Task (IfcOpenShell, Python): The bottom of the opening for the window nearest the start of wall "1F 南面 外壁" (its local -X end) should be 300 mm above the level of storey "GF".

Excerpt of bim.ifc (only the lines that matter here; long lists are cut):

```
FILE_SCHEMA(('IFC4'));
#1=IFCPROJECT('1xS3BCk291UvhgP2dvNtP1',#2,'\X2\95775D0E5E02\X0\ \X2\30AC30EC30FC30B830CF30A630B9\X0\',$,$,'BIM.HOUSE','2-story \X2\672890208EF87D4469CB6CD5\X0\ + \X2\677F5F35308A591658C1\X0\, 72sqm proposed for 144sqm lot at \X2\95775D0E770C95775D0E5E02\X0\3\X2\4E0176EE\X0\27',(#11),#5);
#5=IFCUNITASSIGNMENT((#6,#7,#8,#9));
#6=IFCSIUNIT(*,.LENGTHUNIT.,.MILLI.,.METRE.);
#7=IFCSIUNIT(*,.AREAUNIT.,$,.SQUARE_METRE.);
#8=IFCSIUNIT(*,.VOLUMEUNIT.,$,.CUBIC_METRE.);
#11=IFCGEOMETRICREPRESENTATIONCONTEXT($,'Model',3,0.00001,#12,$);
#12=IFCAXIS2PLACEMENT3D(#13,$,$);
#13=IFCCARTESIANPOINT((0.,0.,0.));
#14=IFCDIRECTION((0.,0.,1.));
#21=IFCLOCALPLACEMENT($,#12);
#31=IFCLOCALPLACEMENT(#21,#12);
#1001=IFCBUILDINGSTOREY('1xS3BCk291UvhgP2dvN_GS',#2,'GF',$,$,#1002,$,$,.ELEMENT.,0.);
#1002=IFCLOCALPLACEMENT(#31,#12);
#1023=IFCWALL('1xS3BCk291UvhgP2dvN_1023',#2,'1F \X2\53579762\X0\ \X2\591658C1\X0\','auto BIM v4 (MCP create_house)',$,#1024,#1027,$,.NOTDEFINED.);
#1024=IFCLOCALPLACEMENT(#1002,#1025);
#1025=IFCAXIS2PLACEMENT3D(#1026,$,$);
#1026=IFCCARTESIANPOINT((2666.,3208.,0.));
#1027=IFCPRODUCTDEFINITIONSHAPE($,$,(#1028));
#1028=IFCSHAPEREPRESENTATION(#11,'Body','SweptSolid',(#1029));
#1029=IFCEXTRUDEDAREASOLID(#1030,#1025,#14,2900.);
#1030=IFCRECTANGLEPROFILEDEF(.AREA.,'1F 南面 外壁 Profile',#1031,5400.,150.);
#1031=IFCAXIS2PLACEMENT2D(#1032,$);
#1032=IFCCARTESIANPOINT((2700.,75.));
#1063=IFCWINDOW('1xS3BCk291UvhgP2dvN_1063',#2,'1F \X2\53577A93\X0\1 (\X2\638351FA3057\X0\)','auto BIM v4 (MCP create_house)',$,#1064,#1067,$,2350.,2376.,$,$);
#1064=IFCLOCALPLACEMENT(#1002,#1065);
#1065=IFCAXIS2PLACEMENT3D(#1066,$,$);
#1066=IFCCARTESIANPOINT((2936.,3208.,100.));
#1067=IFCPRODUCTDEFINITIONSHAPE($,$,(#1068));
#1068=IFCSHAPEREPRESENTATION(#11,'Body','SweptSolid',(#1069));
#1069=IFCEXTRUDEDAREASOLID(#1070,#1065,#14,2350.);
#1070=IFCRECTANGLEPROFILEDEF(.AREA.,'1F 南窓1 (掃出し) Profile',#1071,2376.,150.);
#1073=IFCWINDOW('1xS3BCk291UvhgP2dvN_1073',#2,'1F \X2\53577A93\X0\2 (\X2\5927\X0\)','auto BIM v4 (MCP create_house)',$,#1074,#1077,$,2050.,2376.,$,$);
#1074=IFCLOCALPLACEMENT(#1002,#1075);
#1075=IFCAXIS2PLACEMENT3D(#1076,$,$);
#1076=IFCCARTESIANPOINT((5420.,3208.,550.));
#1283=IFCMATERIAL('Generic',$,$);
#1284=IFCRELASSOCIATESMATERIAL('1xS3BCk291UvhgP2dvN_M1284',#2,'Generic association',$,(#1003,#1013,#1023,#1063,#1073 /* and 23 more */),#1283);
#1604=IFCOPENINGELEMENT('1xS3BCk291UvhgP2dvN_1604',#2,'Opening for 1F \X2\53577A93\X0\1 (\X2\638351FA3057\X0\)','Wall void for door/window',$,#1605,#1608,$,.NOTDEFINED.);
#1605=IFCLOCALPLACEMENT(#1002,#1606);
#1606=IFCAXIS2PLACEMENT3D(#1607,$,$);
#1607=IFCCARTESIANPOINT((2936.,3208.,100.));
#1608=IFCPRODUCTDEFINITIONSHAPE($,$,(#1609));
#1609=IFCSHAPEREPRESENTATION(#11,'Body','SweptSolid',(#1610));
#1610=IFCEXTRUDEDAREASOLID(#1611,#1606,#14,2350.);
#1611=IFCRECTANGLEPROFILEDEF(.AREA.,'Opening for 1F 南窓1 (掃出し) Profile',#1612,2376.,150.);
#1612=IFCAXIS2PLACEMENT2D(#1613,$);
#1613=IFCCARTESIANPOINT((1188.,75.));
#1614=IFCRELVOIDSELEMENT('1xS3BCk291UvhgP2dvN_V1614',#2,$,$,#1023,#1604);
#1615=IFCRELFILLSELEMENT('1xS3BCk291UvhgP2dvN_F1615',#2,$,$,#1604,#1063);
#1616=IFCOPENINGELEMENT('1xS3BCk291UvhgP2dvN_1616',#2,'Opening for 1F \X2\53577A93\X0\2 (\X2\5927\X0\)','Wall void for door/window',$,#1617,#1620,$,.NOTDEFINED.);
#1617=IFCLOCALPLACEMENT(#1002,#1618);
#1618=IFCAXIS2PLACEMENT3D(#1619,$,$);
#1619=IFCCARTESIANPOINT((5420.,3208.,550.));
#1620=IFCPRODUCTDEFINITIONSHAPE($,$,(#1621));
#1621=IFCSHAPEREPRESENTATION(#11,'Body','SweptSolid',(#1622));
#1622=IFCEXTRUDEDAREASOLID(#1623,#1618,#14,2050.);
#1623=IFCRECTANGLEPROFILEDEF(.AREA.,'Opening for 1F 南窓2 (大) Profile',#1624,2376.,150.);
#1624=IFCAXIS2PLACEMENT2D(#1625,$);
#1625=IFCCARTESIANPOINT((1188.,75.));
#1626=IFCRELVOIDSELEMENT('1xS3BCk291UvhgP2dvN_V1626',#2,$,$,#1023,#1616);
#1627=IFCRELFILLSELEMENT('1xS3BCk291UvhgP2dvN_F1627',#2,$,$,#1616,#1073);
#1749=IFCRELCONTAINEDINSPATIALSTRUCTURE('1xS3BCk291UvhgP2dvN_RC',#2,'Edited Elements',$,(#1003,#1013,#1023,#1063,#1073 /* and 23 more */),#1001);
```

```python
import numpy as np
import ifcopenshell
import ifcopenshell.api.geometry
import ifcopenshell.geom
import ifcopenshell.util.element
import ifcopenshell.util.placement
import ifcopenshell.util.shape
import ifcopenshell.util.unit

model = ifcopenshell.open("bim.ifc")
unit_scale = ifcopenshell.util.unit.calculate_unit_scale(model)

window = model.by_guid("1xS3BCk291UvhgP2dvN_1063")
opening = window.FillsVoids[0].RelatingOpeningElement
storey = ifcopenshell.util.element.get_container(window, ifc_class="IfcBuildingStorey")
level = ifcopenshell.util.placement.get_local_placement(storey.ObjectPlacement)[2, 3]

# The opening's origin need not be at the sill, so measure its lowest point.
shape = ifcopenshell.geom.create_shape(ifcopenshell.geom.settings(), opening)
bottom = ifcopenshell.util.shape.get_shape_bottom_elevation(shape, shape.geometry) / unit_scale
dz = level + 0.3 / unit_scale - bottom

shift = np.array([0.0, 0.0, dz])
# The window is not placed relative to its opening, so move both.
for product in (opening, window):
    matrix = ifcopenshell.util.placement.get_local_placement(product.ObjectPlacement)
    matrix[:3, 3] += shift
    ifcopenshell.api.geometry.edit_object_placement(model, product=product, matrix=matrix, is_si=False)

print(f"moved by {dz * unit_scale:+.3f} m")

model.write("bim_edited.ifc")
```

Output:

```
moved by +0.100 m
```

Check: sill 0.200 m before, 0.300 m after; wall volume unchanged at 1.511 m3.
